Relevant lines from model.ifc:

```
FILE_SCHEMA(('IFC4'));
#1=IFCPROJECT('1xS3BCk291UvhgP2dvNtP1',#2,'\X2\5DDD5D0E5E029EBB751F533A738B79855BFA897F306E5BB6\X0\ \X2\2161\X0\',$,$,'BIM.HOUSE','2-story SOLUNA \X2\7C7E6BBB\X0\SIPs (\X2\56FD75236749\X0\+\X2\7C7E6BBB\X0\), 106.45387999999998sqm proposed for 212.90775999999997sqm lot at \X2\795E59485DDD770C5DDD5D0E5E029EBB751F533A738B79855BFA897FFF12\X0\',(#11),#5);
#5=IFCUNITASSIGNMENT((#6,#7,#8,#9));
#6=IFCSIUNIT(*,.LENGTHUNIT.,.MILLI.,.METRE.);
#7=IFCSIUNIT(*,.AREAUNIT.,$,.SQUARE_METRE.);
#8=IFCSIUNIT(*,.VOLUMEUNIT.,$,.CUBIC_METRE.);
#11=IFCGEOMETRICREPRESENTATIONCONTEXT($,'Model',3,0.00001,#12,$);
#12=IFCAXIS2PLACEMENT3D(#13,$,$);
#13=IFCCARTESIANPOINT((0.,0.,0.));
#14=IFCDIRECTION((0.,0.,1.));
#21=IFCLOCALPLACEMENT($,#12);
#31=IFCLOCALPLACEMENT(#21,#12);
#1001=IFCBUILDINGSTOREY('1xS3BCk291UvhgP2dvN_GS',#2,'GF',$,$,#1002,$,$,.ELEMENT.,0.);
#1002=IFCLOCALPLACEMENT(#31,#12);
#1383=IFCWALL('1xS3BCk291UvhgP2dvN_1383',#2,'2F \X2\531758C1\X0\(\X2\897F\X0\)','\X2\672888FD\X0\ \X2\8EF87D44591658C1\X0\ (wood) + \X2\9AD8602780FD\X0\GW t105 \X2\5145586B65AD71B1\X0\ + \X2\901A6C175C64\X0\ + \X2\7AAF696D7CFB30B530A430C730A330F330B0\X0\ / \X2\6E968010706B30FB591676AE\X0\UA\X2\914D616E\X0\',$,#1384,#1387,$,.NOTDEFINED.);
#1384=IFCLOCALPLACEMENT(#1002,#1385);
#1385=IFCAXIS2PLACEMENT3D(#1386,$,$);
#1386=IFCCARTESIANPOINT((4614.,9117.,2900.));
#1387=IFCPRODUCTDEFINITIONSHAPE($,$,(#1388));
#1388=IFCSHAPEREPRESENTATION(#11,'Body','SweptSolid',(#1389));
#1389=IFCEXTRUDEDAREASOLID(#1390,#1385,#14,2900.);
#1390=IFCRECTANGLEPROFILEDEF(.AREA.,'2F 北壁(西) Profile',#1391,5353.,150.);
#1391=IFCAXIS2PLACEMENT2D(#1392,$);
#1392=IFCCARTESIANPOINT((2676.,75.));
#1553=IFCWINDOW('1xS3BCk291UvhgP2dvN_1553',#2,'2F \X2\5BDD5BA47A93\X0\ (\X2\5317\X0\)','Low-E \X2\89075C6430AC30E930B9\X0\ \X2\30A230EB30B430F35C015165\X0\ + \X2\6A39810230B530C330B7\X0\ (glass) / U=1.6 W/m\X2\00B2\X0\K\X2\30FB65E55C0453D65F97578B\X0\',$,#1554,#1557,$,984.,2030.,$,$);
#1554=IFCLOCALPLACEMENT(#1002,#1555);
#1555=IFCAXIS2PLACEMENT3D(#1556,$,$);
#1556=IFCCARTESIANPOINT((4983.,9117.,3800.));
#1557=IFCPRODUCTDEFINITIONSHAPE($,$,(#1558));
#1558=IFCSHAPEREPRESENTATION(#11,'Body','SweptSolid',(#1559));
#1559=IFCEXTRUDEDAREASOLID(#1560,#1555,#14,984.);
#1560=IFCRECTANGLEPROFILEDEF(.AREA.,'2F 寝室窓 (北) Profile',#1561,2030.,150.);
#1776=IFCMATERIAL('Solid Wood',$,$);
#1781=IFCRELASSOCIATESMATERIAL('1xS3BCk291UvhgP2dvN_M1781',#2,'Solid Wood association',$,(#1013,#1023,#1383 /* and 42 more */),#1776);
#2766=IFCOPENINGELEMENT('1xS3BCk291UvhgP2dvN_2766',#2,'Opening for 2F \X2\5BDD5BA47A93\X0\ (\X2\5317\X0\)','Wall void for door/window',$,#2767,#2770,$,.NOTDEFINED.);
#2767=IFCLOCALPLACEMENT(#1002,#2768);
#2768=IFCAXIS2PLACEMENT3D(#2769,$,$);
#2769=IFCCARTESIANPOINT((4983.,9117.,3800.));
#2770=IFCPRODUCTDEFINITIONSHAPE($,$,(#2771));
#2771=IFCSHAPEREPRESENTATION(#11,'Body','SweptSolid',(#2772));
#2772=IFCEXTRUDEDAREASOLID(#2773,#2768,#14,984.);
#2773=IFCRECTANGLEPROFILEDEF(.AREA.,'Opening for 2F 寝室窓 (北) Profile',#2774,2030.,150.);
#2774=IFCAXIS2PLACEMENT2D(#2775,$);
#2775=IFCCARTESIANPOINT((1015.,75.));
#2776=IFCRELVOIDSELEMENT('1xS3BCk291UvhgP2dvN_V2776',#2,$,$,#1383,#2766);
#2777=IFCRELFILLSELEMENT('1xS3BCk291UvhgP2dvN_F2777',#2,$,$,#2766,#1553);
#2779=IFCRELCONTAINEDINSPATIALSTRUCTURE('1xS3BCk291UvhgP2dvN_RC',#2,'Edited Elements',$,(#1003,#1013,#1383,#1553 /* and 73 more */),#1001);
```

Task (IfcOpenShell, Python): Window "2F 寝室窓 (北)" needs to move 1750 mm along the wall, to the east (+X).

```python
import ifcopenshell
import ifcopenshell.api.geometry
import ifcopenshell.util.placement
import ifcopenshell.util.unit

model = ifcopenshell.open("model.ifc")
unit_scale = ifcopenshell.util.unit.calculate_unit_scale(model)

window = model.by_guid("1xS3BCk291UvhgP2dvN_1553")
opening = window.FillsVoids[0].RelatingOpeningElement
wall = opening.VoidsElements[0].RelatingBuildingElement

wall_matrix = ifcopenshell.util.placement.get_local_placement(wall.ObjectPlacement)
shift = wall_matrix[:3, 0] * 1.75 / unit_scale
before = ifcopenshell.util.placement.get_local_placement(window.ObjectPlacement)[:3, 3].copy()

# The window is not placed relative to its opening, so move both.
for product in (opening, window):
    matrix = ifcopenshell.util.placement.get_local_placement(product.ObjectPlacement)
    matrix[:3, 3] += shift
    ifcopenshell.api.geometry.edit_object_placement(model, product=product, matrix=matrix, is_si=False)

after = ifcopenshell.util.placement.get_local_placement(window.ObjectPlacement)[:3, 3]
print("window moved by", (after - before).round(3) + 0.0)

model.write("model_rev.ifc")
```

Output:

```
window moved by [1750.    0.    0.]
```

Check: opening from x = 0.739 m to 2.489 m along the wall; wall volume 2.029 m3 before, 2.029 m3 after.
